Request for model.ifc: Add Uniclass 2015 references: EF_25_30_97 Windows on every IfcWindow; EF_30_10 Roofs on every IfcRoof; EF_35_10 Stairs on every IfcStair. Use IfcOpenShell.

First a look at what the model holds.

```python
import ifcopenshell

model = ifcopenshell.open("model.ifc")
print(model.schema)
print("classifications:", [c.Name for c in model.by_type("IfcClassification")])
for ifc_class in ("IfcDoor", "IfcRoof", "IfcStair", "IfcWall", "IfcWindow"):
    print(ifc_class, len(model.by_type(ifc_class)))
```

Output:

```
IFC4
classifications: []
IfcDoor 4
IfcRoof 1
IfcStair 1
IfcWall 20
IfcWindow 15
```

```python
import ifcopenshell
import ifcopenshell.api.classification

model = ifcopenshell.open("model.ifc")

system = ifcopenshell.api.classification.add_classification(model, classification="Uniclass 2015")

codes = {
    "IfcWindow": ("EF_25_30_97", "Windows"),
    "IfcRoof": ("EF_30_10", "Roofs"),
    "IfcStair": ("EF_35_10", "Stairs"),
}
for ifc_class, (code, name) in codes.items():
    products = model.by_type(ifc_class)
    ifcopenshell.api.classification.add_reference(
        model, products=products, classification=system, identification=code, name=name
    )
    print(code, len(products))

model.write("model-out.ifc")
```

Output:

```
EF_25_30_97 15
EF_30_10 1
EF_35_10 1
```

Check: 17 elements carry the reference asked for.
